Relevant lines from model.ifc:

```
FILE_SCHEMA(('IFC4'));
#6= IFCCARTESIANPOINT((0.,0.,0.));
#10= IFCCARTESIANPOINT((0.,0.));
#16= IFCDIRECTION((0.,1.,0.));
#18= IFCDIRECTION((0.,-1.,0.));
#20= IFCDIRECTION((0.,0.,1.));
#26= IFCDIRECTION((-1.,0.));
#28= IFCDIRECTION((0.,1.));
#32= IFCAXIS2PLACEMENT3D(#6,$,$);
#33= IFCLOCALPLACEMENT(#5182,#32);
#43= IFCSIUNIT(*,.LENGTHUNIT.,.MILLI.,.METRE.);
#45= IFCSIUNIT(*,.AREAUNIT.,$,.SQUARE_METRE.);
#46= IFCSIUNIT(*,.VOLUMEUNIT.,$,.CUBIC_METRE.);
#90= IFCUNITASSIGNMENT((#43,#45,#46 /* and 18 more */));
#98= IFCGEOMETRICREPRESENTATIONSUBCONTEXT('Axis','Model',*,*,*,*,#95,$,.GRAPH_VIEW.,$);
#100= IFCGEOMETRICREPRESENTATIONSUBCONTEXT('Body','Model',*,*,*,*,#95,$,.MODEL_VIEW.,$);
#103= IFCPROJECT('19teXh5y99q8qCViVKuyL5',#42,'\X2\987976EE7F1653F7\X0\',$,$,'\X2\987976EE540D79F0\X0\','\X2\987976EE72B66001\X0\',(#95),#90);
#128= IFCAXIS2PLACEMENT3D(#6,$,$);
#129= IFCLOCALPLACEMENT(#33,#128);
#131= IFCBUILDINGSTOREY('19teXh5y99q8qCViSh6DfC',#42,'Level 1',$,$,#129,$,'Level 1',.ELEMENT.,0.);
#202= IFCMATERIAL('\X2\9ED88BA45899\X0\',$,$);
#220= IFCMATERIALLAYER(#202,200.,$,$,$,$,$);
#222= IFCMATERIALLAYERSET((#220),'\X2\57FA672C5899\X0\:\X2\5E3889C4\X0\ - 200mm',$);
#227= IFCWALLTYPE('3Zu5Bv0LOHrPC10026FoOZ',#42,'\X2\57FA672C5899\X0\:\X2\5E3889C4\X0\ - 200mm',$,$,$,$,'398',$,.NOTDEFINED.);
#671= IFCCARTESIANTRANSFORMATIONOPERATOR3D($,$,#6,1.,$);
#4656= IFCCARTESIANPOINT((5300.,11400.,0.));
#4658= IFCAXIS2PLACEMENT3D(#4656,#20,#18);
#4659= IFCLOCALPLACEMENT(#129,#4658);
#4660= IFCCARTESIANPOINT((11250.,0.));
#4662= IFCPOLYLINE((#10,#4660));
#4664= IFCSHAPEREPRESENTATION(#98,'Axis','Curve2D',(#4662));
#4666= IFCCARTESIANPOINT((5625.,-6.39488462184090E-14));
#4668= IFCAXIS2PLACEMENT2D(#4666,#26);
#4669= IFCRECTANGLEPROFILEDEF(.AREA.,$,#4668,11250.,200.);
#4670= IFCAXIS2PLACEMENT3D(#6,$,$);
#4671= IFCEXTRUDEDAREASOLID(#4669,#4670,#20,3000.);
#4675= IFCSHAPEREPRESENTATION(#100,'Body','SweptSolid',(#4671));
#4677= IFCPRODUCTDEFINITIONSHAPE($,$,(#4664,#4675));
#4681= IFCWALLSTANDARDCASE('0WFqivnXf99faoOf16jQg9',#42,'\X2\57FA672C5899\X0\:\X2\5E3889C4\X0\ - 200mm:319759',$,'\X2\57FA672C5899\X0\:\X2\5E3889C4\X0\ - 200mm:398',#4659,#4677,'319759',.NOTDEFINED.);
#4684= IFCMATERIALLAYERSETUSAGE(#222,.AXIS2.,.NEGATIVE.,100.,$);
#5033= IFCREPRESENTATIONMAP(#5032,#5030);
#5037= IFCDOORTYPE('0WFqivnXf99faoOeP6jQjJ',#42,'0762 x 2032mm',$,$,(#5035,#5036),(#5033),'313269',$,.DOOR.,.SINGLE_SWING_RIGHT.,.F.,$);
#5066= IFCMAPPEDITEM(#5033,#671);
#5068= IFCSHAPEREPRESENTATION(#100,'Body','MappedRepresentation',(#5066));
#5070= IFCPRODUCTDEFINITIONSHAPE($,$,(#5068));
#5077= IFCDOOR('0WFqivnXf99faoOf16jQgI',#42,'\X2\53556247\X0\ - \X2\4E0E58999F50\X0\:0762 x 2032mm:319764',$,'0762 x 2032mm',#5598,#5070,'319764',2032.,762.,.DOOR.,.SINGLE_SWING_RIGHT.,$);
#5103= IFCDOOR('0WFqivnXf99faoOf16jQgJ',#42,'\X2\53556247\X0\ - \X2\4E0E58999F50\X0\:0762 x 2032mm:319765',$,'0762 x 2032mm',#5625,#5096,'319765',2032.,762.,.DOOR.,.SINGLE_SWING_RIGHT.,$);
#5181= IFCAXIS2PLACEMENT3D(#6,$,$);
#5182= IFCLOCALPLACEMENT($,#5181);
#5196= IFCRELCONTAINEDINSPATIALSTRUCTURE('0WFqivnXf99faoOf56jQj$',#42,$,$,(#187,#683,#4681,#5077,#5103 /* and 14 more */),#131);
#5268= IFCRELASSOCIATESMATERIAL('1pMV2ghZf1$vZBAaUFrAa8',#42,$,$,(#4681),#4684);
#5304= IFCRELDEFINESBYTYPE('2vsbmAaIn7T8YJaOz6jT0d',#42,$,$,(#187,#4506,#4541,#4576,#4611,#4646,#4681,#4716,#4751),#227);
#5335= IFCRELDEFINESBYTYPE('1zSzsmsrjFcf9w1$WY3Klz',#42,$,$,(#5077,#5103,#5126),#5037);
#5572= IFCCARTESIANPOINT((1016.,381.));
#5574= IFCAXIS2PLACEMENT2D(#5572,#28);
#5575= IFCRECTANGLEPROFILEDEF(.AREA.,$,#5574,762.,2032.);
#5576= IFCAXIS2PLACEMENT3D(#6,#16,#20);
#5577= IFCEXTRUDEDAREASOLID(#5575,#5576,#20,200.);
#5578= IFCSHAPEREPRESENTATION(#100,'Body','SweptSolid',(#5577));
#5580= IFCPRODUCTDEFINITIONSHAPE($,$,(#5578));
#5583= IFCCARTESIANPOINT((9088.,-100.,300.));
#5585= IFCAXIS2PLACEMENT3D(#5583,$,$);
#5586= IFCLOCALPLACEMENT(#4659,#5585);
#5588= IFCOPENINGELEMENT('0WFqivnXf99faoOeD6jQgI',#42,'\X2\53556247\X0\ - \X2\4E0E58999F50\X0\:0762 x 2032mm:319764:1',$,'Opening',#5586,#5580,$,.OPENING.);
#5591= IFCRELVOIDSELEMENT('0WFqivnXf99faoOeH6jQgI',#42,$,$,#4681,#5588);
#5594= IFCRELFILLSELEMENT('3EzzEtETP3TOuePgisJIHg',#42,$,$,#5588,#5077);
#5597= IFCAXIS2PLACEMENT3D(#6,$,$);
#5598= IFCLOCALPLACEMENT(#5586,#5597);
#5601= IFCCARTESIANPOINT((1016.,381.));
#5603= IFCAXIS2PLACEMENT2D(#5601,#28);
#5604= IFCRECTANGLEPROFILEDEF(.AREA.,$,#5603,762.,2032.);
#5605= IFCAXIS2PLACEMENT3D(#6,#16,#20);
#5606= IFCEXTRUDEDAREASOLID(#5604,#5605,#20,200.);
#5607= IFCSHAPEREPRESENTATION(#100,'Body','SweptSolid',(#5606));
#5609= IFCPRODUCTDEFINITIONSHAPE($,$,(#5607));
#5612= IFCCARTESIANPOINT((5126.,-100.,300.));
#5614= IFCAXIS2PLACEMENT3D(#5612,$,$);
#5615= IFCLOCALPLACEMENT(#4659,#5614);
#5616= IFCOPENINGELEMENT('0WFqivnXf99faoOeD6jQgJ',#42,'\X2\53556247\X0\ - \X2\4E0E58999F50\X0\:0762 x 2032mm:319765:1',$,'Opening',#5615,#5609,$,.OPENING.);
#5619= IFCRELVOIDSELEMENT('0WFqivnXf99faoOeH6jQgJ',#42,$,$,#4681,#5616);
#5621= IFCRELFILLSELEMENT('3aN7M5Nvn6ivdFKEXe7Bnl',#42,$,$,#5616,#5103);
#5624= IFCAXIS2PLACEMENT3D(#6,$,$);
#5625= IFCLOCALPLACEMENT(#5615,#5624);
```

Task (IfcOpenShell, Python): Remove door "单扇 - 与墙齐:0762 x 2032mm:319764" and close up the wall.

```python
import ifcopenshell
import ifcopenshell.api.feature
import ifcopenshell.api.root
import ifcopenshell.geom
import ifcopenshell.util.shape

model = ifcopenshell.open("model.ifc")
settings = ifcopenshell.geom.settings()


def volume(element):
    """Net volume in cubic metres, openings subtracted."""
    shape = ifcopenshell.geom.create_shape(settings, element)
    return ifcopenshell.util.shape.get_volume(shape.geometry)


door = model.by_guid("0WFqivnXf99faoOf16jQgI")
opening = door.FillsVoids[0].RelatingOpeningElement
wall = opening.VoidsElements[0].RelatingBuildingElement
before = volume(wall)

ifcopenshell.api.root.remove_product(model, product=door)
ifcopenshell.api.feature.remove_feature(model, feature=opening)

after = volume(wall)

print(f"wall volume {before:.3f} -> {after:.3f} m3")

model.write("model-out.ifc")
```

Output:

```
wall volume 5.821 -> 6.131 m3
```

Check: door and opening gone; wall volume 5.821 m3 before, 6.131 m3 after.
